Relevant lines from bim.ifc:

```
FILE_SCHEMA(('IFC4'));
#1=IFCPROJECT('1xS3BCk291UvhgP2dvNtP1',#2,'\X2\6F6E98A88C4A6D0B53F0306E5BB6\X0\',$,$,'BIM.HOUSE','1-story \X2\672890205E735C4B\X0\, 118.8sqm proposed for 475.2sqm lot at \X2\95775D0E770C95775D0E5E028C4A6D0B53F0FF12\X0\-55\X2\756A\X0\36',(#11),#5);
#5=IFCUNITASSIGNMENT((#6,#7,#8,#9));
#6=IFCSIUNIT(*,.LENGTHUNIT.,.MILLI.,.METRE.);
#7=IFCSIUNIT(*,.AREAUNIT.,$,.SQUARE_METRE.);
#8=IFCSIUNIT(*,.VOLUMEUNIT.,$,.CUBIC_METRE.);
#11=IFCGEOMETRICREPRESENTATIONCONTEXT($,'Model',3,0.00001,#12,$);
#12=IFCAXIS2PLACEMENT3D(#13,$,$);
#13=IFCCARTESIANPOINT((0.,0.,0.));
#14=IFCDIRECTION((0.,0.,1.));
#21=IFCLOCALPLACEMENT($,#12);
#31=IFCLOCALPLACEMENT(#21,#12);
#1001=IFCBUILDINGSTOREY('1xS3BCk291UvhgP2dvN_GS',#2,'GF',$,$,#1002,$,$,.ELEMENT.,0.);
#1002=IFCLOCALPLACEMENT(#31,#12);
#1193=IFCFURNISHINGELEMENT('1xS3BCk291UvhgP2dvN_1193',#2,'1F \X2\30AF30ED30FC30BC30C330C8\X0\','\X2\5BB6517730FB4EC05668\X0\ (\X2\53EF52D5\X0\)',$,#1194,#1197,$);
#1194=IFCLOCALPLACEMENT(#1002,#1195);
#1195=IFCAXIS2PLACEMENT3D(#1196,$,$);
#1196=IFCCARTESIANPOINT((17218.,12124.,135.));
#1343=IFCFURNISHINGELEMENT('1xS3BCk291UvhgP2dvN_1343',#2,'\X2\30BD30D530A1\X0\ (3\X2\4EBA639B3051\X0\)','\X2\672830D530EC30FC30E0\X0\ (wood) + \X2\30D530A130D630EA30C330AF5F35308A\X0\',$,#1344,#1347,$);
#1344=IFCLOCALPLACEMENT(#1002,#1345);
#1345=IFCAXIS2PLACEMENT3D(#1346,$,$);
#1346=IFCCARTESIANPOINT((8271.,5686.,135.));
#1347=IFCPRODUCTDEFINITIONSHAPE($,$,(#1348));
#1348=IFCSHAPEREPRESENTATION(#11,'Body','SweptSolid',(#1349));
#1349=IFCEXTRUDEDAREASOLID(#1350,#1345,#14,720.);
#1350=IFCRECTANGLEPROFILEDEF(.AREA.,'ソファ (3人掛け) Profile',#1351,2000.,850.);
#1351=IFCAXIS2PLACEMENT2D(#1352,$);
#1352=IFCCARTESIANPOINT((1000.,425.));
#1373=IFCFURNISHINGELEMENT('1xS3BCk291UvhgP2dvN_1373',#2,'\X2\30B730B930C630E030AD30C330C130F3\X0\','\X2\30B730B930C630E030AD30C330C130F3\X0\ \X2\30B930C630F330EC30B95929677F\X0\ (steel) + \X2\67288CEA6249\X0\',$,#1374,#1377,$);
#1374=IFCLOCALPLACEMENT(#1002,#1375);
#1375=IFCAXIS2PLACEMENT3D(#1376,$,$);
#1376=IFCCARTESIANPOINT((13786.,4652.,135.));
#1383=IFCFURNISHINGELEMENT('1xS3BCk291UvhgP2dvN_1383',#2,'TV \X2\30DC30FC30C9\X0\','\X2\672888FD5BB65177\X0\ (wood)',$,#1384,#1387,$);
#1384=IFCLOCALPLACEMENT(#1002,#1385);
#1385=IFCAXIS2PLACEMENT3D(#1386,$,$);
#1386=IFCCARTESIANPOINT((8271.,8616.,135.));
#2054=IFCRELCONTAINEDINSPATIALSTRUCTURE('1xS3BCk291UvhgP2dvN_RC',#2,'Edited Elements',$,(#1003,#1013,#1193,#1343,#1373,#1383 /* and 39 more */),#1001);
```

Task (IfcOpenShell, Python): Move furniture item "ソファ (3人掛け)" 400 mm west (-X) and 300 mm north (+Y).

```python
import ifcopenshell
import ifcopenshell.api.geometry
import ifcopenshell.util.placement

model = ifcopenshell.open("bim.ifc")

item = model.by_id(1343)
matrix = ifcopenshell.util.placement.get_local_placement(item.ObjectPlacement)
matrix[0, 3] -= 400.0
matrix[1, 3] += 300.0
ifcopenshell.api.geometry.edit_object_placement(model, product=item, matrix=matrix, is_si=False)

print(ifcopenshell.util.placement.get_local_placement(item.ObjectPlacement).round(3) + 0.0)

model.write("bim-out.ifc")
```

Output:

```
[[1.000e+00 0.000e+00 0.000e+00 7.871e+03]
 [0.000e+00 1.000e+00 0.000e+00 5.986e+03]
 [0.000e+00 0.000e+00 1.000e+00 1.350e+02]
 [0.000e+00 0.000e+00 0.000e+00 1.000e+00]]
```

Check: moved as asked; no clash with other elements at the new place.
